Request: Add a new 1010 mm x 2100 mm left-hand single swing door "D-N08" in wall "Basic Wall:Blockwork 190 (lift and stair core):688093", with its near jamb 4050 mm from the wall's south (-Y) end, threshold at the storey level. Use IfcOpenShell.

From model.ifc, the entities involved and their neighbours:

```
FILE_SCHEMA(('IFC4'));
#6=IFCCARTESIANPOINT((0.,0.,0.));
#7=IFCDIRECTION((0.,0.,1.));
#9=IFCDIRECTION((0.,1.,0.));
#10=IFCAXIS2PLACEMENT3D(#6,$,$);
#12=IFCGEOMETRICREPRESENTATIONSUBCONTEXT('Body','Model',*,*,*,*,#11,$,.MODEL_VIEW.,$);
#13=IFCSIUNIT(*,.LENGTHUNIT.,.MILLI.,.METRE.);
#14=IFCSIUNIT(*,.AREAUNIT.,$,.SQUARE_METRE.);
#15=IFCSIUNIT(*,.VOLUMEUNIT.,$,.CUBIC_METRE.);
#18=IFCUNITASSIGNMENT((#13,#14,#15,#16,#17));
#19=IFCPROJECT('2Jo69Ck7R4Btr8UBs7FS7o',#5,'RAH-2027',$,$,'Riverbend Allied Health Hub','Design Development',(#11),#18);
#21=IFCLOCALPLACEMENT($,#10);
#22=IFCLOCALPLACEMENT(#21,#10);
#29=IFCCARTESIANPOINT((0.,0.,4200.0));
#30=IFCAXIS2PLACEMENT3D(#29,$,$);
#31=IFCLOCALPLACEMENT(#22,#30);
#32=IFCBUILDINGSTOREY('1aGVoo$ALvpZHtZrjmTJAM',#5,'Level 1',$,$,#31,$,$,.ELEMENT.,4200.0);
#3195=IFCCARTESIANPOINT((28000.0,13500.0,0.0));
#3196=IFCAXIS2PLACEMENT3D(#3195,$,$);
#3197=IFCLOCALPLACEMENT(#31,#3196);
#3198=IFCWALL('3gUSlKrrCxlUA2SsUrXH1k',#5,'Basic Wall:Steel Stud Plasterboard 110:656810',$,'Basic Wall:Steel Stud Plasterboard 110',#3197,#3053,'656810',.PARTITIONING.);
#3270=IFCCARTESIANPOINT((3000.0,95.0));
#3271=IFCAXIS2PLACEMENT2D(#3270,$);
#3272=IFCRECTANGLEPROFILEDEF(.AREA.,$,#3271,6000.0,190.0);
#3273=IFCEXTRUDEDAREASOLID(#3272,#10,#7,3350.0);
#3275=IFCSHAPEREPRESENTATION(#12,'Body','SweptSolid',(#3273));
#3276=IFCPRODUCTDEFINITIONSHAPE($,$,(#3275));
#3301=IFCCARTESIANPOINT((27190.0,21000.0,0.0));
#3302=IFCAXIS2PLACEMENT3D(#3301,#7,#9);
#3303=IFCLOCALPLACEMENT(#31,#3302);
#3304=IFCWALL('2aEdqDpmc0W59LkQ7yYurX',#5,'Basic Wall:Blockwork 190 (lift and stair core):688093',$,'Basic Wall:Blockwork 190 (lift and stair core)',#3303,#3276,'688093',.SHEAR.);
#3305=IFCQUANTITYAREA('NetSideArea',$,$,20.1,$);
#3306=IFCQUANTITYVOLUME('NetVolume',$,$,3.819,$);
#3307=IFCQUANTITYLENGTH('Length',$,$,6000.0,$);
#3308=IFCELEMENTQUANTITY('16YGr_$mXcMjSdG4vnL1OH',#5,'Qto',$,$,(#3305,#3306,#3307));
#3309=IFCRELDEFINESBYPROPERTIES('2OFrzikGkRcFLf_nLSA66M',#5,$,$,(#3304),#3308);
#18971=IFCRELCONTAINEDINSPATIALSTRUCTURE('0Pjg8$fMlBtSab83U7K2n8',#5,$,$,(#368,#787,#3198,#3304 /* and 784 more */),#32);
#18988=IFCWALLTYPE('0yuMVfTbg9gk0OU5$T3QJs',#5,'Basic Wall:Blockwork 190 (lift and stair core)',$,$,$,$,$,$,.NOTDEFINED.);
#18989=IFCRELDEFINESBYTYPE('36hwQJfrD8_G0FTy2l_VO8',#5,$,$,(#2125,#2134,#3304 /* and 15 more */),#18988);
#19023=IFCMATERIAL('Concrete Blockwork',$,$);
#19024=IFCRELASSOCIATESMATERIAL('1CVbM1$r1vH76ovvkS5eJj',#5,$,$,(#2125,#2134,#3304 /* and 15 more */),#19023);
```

```python
import numpy as np
import ifcopenshell
import ifcopenshell.api.feature
import ifcopenshell.api.geometry
import ifcopenshell.api.pset
import ifcopenshell.api.root
import ifcopenshell.api.spatial
import ifcopenshell.geom
import ifcopenshell.util.element
import ifcopenshell.util.placement
import ifcopenshell.util.representation
import ifcopenshell.util.shape
import ifcopenshell.util.unit

model = ifcopenshell.open("model.ifc")
unit_scale = ifcopenshell.util.unit.calculate_unit_scale(model)
area_scale = ifcopenshell.util.unit.calculate_unit_scale(model, "AREAUNIT")
volume_scale = ifcopenshell.util.unit.calculate_unit_scale(model, "VOLUMEUNIT")
settings = ifcopenshell.geom.settings()


def volume(element):
    """Net volume in cubic metres, openings subtracted."""
    shape = ifcopenshell.geom.create_shape(settings, element)
    return ifcopenshell.util.shape.get_volume(shape.geometry)


wall = model.by_id(3304)
storey = ifcopenshell.util.element.get_container(wall, ifc_class="IfcBuildingStorey")
context = ifcopenshell.util.representation.get_context(model, "Model", "Body", "MODEL_VIEW")
before = volume(wall)

width, height, from_end, sill = 1.01, 2.1, 4.05, 0.0  # metres

# The wall runs along its own X axis, and the end named is its -X end.
wall_shape = ifcopenshell.geom.create_shape(settings, wall)
x, y, z = ifcopenshell.util.shape.get_vertices(wall_shape.geometry).T
start = x.min() + from_end
face, thickness = float(y.min()), float(y.max() - y.min())
wall_matrix = ifcopenshell.util.placement.get_local_placement(wall.ObjectPlacement)
level = ifcopenshell.util.placement.get_local_placement(storey.ObjectPlacement)[2, 3]


def in_wall(x, y):
    """Placement at x, y metres in the wall's axes, at sill height."""
    matrix = wall_matrix.copy()
    matrix[:, 3] = wall_matrix @ np.array([x / unit_scale, y / unit_scale, 0.0, 1.0])
    matrix[2, 3] = level + sill / unit_scale
    return matrix


# Opening: a box that overshoots both wall faces by 50 mm.
opening = ifcopenshell.api.root.create_entity(model, ifc_class="IfcOpeningElement", predefined_type="OPENING")
box = ifcopenshell.api.geometry.add_wall_representation(
    model, context=context, length=width, height=height, thickness=thickness + 0.1
)
ifcopenshell.api.geometry.assign_representation(model, product=opening, representation=box)
ifcopenshell.api.geometry.edit_object_placement(model, product=opening, matrix=in_wall(start, face - 0.05), is_si=False)
ifcopenshell.api.feature.add_feature(model, feature=opening, element=wall)

door = ifcopenshell.api.root.create_entity(model, ifc_class="IfcDoor", name="D-N08", predefined_type="DOOR")
door.OverallWidth, door.OverallHeight = width / unit_scale, height / unit_scale
door.OperationType = "SINGLE_SWING_LEFT"
body = ifcopenshell.api.geometry.add_door_representation(
    model,
    context=context,
    overall_width=door.OverallWidth,
    overall_height=door.OverallHeight,
    operation_type="SINGLE_SWING_LEFT",
    lining_properties={"LiningDepth": thickness / unit_scale, "ThresholdDepth": thickness / unit_scale},
)
ifcopenshell.api.geometry.assign_representation(model, product=door, representation=body)
ifcopenshell.api.spatial.assign_container(model, products=[door], relating_structure=storey)
ifcopenshell.api.feature.add_filling(model, opening=opening, element=door)

# The lining spans the wall, so the door starts at the wall face.
ifcopenshell.api.geometry.edit_object_placement(model, product=door, matrix=in_wall(start, face), is_si=False)

after = volume(wall)

# Update the wall's stored quantities.
qto = model.by_id(ifcopenshell.util.element.get_pset(wall, "Qto", should_inherit=False)["id"])
ifcopenshell.api.pset.edit_qto(model, qto=qto, properties={
    "NetSideArea": after / thickness / area_scale,
    "NetVolume": after / volume_scale,
})

print(f"wall volume {before:.3f} -> {after:.3f} m3")

model.write("model_v2.ifc")
```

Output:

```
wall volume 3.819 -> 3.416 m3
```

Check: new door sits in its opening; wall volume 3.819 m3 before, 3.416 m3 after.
